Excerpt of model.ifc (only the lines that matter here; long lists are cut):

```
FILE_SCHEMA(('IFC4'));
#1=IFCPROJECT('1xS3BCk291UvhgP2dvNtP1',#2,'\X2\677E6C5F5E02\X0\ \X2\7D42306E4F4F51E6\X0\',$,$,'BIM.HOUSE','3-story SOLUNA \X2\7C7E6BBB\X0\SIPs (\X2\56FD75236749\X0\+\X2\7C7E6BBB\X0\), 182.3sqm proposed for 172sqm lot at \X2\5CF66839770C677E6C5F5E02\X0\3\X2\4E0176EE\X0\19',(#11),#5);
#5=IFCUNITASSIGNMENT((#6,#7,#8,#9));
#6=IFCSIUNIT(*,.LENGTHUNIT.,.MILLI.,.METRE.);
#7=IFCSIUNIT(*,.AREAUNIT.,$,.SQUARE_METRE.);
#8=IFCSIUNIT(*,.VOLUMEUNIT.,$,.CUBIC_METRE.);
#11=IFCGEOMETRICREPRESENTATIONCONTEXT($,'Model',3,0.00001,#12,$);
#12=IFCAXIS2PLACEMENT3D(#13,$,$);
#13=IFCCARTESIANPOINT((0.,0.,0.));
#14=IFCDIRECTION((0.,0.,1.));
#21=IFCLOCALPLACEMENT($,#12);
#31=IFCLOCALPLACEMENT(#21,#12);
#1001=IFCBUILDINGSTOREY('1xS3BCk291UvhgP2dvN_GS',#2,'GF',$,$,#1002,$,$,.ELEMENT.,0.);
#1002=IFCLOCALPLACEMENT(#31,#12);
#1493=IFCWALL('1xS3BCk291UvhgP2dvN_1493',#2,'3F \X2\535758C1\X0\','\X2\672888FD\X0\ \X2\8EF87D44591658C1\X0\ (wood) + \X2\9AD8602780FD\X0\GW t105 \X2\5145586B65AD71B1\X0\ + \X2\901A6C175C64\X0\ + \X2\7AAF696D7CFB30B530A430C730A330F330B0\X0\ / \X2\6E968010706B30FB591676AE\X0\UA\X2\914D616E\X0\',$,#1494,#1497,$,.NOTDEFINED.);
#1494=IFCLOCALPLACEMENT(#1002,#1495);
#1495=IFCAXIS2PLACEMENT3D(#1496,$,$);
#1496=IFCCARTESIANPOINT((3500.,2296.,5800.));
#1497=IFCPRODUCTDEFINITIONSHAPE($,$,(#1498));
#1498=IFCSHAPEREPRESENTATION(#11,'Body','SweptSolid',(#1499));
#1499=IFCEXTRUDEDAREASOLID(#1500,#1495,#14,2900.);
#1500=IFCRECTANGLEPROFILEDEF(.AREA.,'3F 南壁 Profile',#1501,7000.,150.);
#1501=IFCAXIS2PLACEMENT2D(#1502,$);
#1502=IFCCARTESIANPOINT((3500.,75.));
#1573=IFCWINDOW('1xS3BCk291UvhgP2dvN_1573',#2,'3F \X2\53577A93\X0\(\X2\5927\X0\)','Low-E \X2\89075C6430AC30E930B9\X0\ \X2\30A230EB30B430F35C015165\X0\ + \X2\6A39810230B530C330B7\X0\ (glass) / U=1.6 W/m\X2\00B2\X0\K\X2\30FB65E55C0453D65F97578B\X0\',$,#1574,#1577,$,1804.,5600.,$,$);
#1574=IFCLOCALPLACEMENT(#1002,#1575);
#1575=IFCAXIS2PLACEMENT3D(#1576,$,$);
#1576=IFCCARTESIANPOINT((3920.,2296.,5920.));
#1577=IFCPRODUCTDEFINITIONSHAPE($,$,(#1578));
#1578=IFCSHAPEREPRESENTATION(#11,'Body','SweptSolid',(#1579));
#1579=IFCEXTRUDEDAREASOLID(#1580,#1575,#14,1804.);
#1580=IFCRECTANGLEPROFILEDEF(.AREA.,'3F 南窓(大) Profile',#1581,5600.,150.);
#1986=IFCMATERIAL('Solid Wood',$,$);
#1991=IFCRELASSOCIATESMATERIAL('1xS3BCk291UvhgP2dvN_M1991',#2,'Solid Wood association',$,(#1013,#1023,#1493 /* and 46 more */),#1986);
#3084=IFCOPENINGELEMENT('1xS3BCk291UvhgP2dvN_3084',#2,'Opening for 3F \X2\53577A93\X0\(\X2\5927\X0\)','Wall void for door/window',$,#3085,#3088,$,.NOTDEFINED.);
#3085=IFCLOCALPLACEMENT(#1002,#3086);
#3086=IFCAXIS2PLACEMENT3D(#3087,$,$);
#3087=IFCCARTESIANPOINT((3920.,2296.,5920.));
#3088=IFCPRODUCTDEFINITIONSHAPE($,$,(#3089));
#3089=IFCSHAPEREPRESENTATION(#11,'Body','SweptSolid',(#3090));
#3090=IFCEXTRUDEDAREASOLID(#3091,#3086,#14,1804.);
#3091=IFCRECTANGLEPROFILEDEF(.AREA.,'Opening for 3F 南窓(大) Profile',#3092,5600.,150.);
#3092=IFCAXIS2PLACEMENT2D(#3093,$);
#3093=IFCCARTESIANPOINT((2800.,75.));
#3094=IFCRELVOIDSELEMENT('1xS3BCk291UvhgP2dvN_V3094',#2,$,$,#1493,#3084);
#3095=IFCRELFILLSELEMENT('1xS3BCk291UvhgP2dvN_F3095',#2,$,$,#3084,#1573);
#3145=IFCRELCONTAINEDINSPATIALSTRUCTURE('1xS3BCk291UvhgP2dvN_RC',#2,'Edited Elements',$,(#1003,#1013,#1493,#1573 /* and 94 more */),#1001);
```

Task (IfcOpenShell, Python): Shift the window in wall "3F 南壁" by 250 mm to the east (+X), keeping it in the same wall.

```python
import ifcopenshell
import ifcopenshell.api.geometry
import ifcopenshell.util.placement
import ifcopenshell.util.unit

model = ifcopenshell.open("model.ifc")
unit_scale = ifcopenshell.util.unit.calculate_unit_scale(model)

window = model.by_id(1573)
opening = window.FillsVoids[0].RelatingOpeningElement
wall = opening.VoidsElements[0].RelatingBuildingElement

wall_matrix = ifcopenshell.util.placement.get_local_placement(wall.ObjectPlacement)
shift = wall_matrix[:3, 0] * 0.25 / unit_scale
before = ifcopenshell.util.placement.get_local_placement(window.ObjectPlacement)[:3, 3].copy()

# The window is not placed relative to its opening, so move both.
for product in (opening, window):
    matrix = ifcopenshell.util.placement.get_local_placement(product.ObjectPlacement)
    matrix[:3, 3] += shift
    ifcopenshell.api.geometry.edit_object_placement(model, product=product, matrix=matrix, is_si=False)

after = ifcopenshell.util.placement.get_local_placement(window.ObjectPlacement)[:3, 3]
print("window moved by", (after - before).round(3) + 0.0)

model.write("model_edited.ifc")
```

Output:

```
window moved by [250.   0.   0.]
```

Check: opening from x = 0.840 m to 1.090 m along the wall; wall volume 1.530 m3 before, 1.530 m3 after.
